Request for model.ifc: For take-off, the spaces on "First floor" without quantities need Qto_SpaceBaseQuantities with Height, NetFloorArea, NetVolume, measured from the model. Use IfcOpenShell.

First a look at what the model holds.

```python
import ifcopenshell
import ifcopenshell.util.element
import ifcopenshell.util.unit

model = ifcopenshell.open("model.ifc")
print(model.schema)
for unit_type in ("LENGTHUNIT", "AREAUNIT", "VOLUMEUNIT"):
    print(unit_type, ifcopenshell.util.unit.calculate_unit_scale(model, unit_type))
storey = next(s for s in model.by_type("IfcBuildingStorey") if s.Name == "First floor")
spaces = [e for e in ifcopenshell.util.element.get_decomposition(storey) if e.is_a("IfcSpace")]
for e in sorted(spaces, key=lambda e: e.id()):
    print(e.id(), e.is_a(), e.Name, list(ifcopenshell.util.element.get_psets(e, qtos_only=True)), sep=" | ")
```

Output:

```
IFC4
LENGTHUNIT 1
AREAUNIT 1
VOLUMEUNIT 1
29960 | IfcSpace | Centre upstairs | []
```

```python
import ifcopenshell
import ifcopenshell.api.pset
import ifcopenshell.geom
import ifcopenshell.util.element
import ifcopenshell.util.shape
import ifcopenshell.util.unit

model = ifcopenshell.open("model.ifc")
unit_scale = ifcopenshell.util.unit.calculate_unit_scale(model)
area_scale = ifcopenshell.util.unit.calculate_unit_scale(model, "AREAUNIT")
volume_scale = ifcopenshell.util.unit.calculate_unit_scale(model, "VOLUMEUNIT")
settings = ifcopenshell.geom.settings()

storey = next(s for s in model.by_type("IfcBuildingStorey") if s.Name == "First floor")
spaces = [e for e in ifcopenshell.util.element.get_decomposition(storey) if e.is_a("IfcSpace")]

for e in sorted(spaces, key=lambda e: e.id()):
    if ifcopenshell.util.element.get_psets(e, qtos_only=True, should_inherit=False):
        continue
    # Geometry comes back in metres, in the element's own axes.
    shape = ifcopenshell.geom.create_shape(settings, e)
    values = {
        "Height": ifcopenshell.util.shape.get_z(shape.geometry) / unit_scale,
        "NetFloorArea": ifcopenshell.util.shape.get_footprint_area(shape.geometry) / area_scale,
        "NetVolume": ifcopenshell.util.shape.get_volume(shape.geometry) / volume_scale,
    }
    qto = ifcopenshell.api.pset.add_qto(model, product=e, name="Qto_SpaceBaseQuantities")
    ifcopenshell.api.pset.edit_qto(model, qto=qto, properties=values)
    print(e.id(), {k: round(v, 3) for k, v in values.items()})

model.write("model_updated.ifc")
```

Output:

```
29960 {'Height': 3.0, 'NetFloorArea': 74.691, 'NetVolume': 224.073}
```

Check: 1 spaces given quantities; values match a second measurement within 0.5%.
